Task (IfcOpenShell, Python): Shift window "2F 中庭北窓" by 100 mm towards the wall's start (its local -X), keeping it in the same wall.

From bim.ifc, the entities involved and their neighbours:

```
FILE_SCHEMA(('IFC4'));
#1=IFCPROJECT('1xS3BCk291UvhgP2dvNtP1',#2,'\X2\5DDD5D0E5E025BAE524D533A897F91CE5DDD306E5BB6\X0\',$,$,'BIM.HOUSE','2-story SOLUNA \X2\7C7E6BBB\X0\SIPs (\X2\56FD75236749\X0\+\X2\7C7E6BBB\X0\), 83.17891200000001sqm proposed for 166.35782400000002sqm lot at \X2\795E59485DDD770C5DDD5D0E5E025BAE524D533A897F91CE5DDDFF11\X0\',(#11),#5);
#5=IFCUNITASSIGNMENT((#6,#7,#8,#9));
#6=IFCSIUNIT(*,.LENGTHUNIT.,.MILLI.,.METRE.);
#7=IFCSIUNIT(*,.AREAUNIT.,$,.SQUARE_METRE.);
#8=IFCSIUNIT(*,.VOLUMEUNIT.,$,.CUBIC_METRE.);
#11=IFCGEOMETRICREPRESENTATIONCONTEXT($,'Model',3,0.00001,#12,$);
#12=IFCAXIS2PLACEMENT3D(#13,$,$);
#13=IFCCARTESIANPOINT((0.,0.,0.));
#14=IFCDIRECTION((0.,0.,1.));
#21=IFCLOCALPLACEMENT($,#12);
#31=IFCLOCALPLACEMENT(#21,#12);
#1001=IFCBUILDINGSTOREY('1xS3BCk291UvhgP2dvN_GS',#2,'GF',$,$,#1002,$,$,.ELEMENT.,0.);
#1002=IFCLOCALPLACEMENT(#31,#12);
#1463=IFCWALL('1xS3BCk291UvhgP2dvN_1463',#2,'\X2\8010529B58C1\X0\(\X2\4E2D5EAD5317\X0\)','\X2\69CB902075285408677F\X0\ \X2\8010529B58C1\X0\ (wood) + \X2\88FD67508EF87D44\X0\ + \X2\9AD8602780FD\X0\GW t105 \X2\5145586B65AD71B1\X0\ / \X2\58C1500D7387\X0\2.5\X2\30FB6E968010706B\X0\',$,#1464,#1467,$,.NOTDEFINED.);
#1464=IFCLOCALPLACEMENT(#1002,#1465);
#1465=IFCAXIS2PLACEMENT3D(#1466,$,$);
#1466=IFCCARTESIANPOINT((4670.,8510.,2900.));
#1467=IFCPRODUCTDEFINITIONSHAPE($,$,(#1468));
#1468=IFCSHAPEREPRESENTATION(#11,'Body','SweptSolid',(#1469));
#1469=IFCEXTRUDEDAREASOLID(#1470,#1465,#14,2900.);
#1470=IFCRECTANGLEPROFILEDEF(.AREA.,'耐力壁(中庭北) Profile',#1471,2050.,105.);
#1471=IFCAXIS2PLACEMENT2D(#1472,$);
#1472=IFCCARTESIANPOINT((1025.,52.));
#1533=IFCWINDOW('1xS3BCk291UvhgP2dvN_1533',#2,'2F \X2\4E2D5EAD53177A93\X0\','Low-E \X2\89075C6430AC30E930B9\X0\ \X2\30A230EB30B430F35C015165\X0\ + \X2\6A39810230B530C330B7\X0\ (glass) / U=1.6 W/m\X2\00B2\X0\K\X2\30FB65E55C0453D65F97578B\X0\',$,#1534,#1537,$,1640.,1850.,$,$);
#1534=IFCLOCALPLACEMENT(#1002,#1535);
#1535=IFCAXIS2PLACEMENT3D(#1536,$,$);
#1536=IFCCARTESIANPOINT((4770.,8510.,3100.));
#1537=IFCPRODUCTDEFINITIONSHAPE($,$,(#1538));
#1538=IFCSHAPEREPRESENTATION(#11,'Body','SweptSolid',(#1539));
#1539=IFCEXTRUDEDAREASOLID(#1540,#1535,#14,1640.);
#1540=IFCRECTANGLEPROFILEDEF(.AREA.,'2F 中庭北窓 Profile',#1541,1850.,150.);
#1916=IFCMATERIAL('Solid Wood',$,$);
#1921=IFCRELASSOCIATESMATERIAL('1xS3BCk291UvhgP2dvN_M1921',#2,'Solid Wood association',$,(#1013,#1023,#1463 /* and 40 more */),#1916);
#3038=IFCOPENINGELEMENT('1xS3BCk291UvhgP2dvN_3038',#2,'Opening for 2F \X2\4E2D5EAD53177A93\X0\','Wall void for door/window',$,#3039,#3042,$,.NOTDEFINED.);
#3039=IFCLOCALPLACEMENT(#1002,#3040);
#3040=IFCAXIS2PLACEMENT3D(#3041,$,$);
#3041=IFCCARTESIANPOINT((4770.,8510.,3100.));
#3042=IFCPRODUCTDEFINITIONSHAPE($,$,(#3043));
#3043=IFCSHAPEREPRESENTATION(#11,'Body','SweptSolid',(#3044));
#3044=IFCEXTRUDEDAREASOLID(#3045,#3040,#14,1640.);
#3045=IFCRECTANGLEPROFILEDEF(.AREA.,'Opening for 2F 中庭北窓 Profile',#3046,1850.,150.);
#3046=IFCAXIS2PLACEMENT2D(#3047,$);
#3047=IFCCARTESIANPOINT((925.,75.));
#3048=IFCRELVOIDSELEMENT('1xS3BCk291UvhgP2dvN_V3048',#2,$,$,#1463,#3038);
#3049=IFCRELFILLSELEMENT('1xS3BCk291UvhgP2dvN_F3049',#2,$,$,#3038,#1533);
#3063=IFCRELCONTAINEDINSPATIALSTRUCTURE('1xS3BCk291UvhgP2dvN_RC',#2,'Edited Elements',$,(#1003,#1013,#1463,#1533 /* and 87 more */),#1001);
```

```python
import ifcopenshell
import ifcopenshell.api.geometry
import ifcopenshell.util.placement
import ifcopenshell.util.unit

model = ifcopenshell.open("bim.ifc")
unit_scale = ifcopenshell.util.unit.calculate_unit_scale(model)

window = model.by_guid("1xS3BCk291UvhgP2dvN_1533")
opening = window.FillsVoids[0].RelatingOpeningElement
wall = opening.VoidsElements[0].RelatingBuildingElement

wall_matrix = ifcopenshell.util.placement.get_local_placement(wall.ObjectPlacement)
shift = wall_matrix[:3, 0] * -0.1 / unit_scale
before = ifcopenshell.util.placement.get_local_placement(window.ObjectPlacement)[:3, 3].copy()

# The window is not placed relative to its opening, so move both.
for product in (opening, window):
    matrix = ifcopenshell.util.placement.get_local_placement(product.ObjectPlacement)
    matrix[:3, 3] += shift
    ifcopenshell.api.geometry.edit_object_placement(model, product=product, matrix=matrix, is_si=False)

after = ifcopenshell.util.placement.get_local_placement(window.ObjectPlacement)[:3, 3]
print("window moved by", (after - before).round(3) + 0.0)

model.write("bim_rev.ifc")
```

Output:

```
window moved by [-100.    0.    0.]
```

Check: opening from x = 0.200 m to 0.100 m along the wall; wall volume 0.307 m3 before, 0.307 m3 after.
